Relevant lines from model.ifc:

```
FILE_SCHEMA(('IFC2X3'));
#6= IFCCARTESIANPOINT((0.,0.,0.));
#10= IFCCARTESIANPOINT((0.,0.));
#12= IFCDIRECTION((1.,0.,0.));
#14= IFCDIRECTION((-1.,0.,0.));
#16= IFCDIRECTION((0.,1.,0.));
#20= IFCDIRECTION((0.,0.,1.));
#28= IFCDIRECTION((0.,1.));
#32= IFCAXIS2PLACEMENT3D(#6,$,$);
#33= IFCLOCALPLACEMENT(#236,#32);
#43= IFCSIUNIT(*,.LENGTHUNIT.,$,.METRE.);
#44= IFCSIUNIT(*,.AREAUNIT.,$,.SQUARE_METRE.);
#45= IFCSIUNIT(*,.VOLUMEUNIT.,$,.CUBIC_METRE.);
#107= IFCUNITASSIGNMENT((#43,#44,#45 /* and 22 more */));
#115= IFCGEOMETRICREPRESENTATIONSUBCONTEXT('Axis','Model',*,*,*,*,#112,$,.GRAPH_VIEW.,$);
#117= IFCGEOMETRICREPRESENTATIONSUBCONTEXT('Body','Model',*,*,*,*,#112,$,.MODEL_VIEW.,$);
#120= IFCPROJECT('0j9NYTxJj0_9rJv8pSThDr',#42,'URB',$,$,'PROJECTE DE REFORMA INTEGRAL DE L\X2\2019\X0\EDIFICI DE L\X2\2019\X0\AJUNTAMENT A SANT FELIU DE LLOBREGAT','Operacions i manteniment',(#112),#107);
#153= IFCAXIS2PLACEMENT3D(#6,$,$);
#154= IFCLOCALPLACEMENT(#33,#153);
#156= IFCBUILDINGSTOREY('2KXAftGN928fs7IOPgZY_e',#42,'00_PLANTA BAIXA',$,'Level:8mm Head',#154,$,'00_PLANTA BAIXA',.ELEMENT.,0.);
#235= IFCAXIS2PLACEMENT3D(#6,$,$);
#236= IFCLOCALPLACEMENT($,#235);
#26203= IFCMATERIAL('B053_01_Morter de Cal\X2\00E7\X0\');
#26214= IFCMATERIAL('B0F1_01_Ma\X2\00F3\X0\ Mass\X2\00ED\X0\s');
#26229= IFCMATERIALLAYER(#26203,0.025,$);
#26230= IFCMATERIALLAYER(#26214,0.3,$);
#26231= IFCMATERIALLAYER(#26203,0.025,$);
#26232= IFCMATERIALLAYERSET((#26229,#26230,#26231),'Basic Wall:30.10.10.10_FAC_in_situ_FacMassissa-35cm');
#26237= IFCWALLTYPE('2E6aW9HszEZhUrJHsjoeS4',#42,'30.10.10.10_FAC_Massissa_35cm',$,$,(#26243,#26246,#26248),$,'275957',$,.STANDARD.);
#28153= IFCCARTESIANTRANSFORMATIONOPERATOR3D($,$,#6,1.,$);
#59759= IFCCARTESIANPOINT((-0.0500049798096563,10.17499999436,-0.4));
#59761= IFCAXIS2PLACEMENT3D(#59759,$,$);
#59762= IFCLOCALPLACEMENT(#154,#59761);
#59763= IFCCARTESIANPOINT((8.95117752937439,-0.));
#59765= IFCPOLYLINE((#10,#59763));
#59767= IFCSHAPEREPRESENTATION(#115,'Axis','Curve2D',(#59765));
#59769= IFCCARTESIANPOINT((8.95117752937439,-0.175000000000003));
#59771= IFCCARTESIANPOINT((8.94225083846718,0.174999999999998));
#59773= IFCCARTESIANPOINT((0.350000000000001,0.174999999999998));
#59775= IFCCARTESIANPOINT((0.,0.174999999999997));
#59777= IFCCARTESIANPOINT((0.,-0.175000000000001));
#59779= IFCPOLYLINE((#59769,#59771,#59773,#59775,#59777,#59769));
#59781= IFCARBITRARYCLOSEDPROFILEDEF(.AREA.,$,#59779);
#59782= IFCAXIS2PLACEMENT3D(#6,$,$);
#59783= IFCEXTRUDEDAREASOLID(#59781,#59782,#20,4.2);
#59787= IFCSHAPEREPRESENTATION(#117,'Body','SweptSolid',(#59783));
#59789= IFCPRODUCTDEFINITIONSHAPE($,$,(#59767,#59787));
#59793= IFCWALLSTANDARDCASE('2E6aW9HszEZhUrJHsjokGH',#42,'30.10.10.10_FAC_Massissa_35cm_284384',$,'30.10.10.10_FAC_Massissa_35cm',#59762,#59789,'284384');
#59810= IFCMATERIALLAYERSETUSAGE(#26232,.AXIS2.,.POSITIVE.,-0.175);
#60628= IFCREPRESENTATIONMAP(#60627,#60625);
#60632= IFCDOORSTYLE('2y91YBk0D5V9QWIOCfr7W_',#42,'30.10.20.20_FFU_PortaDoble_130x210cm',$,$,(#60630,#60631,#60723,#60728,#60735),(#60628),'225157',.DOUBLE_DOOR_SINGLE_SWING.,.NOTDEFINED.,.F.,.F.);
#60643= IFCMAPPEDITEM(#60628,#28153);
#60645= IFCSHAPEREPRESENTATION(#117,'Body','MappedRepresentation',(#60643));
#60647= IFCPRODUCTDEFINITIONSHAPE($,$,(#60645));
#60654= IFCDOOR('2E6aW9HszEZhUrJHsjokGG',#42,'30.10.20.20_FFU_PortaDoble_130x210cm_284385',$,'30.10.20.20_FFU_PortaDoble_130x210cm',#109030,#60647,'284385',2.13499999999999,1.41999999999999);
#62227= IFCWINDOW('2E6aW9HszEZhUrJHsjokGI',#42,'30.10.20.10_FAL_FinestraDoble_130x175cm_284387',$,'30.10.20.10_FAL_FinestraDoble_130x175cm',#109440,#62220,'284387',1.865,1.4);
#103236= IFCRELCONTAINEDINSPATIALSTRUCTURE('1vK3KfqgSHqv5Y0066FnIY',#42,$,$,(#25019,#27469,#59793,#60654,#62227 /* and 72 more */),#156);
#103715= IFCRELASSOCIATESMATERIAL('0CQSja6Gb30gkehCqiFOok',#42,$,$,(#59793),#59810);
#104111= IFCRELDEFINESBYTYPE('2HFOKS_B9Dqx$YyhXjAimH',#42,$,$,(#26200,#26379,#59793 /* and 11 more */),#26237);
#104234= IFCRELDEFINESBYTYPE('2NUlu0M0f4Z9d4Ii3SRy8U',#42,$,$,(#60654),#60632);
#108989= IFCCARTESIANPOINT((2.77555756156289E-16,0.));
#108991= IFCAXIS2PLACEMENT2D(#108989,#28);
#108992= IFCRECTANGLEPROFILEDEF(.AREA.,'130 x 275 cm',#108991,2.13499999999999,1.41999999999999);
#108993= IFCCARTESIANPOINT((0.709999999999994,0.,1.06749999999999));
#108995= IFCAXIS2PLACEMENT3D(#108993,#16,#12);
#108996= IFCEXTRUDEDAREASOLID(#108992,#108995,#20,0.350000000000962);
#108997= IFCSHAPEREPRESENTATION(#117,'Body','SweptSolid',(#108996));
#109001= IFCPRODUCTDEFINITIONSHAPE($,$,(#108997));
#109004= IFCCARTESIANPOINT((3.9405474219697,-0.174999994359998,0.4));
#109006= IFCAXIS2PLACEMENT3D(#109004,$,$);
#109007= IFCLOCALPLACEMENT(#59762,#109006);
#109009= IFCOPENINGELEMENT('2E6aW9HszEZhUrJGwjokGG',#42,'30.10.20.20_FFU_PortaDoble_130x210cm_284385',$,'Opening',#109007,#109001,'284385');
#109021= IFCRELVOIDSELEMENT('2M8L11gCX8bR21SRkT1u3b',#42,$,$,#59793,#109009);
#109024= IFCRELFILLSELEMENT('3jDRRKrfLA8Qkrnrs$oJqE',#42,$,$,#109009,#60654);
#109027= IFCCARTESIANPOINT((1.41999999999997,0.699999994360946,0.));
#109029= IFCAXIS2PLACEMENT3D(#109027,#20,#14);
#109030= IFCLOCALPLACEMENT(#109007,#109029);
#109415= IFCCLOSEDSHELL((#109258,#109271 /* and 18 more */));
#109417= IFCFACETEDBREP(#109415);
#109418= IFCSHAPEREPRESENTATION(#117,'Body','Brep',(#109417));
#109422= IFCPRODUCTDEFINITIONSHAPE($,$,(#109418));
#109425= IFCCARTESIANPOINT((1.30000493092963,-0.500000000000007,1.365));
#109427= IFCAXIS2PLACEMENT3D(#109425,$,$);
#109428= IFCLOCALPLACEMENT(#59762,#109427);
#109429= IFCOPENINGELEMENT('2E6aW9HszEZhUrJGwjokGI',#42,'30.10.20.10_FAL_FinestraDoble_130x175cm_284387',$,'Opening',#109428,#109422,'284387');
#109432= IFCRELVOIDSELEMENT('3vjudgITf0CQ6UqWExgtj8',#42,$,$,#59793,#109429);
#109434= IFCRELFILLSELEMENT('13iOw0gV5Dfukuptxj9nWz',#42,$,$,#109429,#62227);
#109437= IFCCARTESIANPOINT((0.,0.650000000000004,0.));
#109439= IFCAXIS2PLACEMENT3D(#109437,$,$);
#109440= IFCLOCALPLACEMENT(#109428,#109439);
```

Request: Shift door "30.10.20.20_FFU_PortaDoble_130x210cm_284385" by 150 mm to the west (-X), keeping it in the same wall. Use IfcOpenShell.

```python
import ifcopenshell
import ifcopenshell.api.geometry
import ifcopenshell.util.placement
import ifcopenshell.util.unit

model = ifcopenshell.open("model.ifc")
unit_scale = ifcopenshell.util.unit.calculate_unit_scale(model)

door = model.by_guid("2E6aW9HszEZhUrJHsjokGG")
opening = door.FillsVoids[0].RelatingOpeningElement
wall = opening.VoidsElements[0].RelatingBuildingElement

wall_matrix = ifcopenshell.util.placement.get_local_placement(wall.ObjectPlacement)
shift = wall_matrix[:3, 0] * -0.15 / unit_scale
before = ifcopenshell.util.placement.get_local_placement(door.ObjectPlacement)[:3, 3].copy()

# The door is placed relative to its opening, so it follows when the opening moves.
matrix = ifcopenshell.util.placement.get_local_placement(opening.ObjectPlacement)
matrix[:3, 3] += shift
ifcopenshell.api.geometry.edit_object_placement(
    model, product=opening, matrix=matrix, is_si=False, should_transform_children=True
)

after = ifcopenshell.util.placement.get_local_placement(door.ObjectPlacement)[:3, 3]
print("door moved by", (after - before).round(3) + 0.0)

model.write("model_v2.ifc")
```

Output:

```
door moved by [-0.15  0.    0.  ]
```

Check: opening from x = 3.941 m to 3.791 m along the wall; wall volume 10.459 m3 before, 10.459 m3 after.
